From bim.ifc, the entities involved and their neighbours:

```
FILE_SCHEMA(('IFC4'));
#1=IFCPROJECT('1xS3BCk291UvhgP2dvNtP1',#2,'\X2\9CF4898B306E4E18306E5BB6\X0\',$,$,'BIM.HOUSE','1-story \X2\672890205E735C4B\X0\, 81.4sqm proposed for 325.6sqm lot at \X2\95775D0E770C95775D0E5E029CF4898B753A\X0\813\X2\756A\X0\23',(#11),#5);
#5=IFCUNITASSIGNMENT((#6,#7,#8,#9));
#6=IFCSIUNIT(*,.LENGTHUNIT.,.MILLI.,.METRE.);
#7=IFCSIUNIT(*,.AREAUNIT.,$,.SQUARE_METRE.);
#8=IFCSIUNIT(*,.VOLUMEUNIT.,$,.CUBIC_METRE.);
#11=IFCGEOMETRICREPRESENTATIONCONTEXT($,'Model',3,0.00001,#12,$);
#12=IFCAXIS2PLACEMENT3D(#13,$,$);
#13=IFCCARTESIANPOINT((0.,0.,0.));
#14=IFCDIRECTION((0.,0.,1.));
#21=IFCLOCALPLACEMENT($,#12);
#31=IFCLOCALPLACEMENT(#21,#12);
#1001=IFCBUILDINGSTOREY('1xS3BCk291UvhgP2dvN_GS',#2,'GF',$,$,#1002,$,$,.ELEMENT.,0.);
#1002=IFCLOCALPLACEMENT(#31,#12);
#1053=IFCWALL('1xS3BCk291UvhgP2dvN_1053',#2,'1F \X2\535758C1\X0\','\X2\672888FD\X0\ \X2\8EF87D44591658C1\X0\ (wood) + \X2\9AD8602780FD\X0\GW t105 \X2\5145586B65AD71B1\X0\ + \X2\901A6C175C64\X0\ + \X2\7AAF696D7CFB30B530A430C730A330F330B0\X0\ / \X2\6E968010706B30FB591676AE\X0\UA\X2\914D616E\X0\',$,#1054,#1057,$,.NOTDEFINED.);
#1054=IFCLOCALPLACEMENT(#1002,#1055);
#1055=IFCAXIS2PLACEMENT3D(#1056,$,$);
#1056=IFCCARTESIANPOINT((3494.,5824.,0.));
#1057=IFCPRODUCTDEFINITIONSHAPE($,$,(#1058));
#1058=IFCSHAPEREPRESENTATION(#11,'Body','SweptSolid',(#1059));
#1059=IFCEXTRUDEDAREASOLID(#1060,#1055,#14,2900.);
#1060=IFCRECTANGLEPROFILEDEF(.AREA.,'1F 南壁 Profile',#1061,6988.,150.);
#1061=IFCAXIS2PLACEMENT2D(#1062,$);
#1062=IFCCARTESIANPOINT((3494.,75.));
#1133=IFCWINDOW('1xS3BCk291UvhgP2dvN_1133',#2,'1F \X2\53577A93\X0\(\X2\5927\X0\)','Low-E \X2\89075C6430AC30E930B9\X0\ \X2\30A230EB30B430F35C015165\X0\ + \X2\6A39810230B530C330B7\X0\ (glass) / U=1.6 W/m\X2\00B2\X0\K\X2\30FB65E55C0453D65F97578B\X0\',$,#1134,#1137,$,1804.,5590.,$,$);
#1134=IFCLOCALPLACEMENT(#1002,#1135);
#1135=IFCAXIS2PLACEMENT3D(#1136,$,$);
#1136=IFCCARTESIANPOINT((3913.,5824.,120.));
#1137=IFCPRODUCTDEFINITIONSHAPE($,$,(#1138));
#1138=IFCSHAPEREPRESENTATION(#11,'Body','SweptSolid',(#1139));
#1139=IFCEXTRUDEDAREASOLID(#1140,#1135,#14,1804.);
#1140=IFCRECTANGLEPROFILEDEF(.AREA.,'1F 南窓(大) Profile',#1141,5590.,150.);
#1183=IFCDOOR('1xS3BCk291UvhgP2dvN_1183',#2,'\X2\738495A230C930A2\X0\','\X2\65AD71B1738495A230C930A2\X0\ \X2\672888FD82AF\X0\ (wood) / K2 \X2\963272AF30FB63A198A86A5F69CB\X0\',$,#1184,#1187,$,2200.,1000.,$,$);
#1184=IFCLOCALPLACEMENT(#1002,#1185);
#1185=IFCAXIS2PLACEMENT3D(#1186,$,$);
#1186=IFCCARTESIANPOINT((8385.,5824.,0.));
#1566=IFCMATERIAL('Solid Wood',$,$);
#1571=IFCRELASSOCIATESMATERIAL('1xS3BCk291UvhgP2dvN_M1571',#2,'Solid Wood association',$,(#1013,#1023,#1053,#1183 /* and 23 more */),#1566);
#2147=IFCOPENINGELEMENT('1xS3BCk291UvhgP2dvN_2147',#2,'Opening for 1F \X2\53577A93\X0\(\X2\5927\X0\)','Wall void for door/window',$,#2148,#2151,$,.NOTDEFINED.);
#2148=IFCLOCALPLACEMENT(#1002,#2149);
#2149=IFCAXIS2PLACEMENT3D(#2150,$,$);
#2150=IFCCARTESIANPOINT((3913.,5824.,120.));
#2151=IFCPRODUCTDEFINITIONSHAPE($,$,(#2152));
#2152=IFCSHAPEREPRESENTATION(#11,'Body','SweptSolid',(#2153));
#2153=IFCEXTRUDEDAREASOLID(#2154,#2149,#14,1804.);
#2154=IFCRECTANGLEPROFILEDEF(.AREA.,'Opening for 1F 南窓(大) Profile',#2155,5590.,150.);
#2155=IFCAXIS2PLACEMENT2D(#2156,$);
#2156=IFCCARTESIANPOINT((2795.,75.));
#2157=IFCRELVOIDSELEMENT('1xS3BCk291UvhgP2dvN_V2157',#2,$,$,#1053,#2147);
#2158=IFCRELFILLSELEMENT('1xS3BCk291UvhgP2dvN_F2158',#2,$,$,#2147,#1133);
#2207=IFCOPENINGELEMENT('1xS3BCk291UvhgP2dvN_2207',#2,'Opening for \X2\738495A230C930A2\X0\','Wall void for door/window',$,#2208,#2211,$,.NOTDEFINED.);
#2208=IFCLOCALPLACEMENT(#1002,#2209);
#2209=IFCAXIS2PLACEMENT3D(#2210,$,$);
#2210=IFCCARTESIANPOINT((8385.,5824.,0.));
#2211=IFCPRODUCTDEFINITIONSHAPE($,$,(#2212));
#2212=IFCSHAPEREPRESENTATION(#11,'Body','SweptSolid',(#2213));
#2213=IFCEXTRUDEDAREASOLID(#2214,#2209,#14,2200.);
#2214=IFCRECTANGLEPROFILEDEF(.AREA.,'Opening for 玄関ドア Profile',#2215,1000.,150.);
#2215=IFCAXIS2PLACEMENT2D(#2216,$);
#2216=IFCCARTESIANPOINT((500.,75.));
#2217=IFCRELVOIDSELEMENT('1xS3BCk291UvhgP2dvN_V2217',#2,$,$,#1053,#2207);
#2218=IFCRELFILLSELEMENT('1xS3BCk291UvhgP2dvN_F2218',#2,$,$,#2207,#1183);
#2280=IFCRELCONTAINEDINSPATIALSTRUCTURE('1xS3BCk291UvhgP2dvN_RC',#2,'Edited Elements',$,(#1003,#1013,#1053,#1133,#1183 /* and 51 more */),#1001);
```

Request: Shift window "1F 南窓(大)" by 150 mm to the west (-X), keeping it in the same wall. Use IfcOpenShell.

```python
import ifcopenshell
import ifcopenshell.api.geometry
import ifcopenshell.util.placement
import ifcopenshell.util.unit

model = ifcopenshell.open("bim.ifc")
unit_scale = ifcopenshell.util.unit.calculate_unit_scale(model)

window = model.by_guid("1xS3BCk291UvhgP2dvN_1133")
opening = window.FillsVoids[0].RelatingOpeningElement
wall = opening.VoidsElements[0].RelatingBuildingElement

wall_matrix = ifcopenshell.util.placement.get_local_placement(wall.ObjectPlacement)
shift = wall_matrix[:3, 0] * -0.15 / unit_scale
before = ifcopenshell.util.placement.get_local_placement(window.ObjectPlacement)[:3, 3].copy()

# The window is not placed relative to its opening, so move both.
for product in (opening, window):
    matrix = ifcopenshell.util.placement.get_local_placement(product.ObjectPlacement)
    matrix[:3, 3] += shift
    ifcopenshell.api.geometry.edit_object_placement(model, product=product, matrix=matrix, is_si=False)

after = ifcopenshell.util.placement.get_local_placement(window.ObjectPlacement)[:3, 3]
print("window moved by", (after - before).round(3) + 0.0)

model.write("bim_rev.ifc")
```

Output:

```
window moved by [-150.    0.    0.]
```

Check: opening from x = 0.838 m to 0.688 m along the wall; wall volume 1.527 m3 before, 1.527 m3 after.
